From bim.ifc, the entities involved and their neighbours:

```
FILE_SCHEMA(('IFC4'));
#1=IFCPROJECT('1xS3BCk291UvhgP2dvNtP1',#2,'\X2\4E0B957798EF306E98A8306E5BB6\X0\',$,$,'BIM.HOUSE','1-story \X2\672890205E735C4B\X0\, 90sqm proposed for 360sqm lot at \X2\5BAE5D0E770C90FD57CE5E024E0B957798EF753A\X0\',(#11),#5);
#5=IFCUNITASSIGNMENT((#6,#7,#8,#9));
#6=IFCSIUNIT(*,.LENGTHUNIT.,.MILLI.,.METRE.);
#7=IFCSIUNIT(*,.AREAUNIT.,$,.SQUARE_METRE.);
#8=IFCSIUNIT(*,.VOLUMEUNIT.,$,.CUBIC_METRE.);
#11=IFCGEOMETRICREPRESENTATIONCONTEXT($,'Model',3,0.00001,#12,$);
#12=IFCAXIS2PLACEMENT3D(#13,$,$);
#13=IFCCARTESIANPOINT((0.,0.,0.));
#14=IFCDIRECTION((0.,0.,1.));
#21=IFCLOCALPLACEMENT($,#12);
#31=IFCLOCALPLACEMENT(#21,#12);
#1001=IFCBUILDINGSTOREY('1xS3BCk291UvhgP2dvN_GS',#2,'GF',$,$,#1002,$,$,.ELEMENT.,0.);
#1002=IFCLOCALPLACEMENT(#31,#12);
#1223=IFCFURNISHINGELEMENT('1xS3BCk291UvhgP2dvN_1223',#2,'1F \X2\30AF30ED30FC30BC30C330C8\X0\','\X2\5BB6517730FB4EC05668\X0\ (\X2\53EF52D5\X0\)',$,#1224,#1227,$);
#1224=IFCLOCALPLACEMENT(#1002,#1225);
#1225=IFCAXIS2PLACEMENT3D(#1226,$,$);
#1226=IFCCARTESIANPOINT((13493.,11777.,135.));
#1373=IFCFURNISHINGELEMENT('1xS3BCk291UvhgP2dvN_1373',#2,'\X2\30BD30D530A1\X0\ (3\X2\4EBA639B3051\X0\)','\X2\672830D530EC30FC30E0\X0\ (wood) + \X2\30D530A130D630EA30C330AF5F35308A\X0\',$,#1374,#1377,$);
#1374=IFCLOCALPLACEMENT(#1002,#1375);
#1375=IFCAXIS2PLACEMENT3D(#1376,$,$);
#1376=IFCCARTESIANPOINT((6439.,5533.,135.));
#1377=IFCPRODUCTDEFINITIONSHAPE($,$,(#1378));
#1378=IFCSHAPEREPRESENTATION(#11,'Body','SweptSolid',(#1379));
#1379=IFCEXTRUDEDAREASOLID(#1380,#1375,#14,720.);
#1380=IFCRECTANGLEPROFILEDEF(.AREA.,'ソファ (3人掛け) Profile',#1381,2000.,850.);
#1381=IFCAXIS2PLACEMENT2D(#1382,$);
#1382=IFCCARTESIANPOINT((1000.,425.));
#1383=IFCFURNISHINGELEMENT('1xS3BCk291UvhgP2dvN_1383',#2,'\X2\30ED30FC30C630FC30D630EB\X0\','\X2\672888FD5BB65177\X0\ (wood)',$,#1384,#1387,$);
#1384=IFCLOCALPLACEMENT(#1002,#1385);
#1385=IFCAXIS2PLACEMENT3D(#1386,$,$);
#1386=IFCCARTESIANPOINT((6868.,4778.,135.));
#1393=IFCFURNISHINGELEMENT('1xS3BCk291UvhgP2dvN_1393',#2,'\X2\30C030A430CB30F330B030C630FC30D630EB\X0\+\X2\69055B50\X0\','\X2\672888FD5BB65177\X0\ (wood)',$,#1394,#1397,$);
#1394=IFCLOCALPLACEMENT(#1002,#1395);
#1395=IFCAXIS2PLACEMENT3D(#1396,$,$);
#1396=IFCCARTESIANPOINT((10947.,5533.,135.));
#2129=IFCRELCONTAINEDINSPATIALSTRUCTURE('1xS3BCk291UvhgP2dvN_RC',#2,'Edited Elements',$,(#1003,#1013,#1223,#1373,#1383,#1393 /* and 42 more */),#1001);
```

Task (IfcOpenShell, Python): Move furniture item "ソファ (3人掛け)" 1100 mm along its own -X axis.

```python
import ifcopenshell
import ifcopenshell.api.geometry
import ifcopenshell.util.placement
import ifcopenshell.util.unit

model = ifcopenshell.open("bim.ifc")
unit_scale = ifcopenshell.util.unit.calculate_unit_scale(model)

item = model.by_id(1373)
matrix = ifcopenshell.util.placement.get_local_placement(item.ObjectPlacement)
matrix[:3, 3] -= matrix[:3, 0] * 1.1 / unit_scale
ifcopenshell.api.geometry.edit_object_placement(model, product=item, matrix=matrix, is_si=False)

print(ifcopenshell.util.placement.get_local_placement(item.ObjectPlacement).round(3) + 0.0)

model.write("bim_updated.ifc")
```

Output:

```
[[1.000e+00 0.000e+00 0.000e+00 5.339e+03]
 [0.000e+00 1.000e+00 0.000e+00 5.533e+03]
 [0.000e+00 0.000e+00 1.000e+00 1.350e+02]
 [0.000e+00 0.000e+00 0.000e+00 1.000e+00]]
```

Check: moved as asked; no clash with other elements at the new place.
